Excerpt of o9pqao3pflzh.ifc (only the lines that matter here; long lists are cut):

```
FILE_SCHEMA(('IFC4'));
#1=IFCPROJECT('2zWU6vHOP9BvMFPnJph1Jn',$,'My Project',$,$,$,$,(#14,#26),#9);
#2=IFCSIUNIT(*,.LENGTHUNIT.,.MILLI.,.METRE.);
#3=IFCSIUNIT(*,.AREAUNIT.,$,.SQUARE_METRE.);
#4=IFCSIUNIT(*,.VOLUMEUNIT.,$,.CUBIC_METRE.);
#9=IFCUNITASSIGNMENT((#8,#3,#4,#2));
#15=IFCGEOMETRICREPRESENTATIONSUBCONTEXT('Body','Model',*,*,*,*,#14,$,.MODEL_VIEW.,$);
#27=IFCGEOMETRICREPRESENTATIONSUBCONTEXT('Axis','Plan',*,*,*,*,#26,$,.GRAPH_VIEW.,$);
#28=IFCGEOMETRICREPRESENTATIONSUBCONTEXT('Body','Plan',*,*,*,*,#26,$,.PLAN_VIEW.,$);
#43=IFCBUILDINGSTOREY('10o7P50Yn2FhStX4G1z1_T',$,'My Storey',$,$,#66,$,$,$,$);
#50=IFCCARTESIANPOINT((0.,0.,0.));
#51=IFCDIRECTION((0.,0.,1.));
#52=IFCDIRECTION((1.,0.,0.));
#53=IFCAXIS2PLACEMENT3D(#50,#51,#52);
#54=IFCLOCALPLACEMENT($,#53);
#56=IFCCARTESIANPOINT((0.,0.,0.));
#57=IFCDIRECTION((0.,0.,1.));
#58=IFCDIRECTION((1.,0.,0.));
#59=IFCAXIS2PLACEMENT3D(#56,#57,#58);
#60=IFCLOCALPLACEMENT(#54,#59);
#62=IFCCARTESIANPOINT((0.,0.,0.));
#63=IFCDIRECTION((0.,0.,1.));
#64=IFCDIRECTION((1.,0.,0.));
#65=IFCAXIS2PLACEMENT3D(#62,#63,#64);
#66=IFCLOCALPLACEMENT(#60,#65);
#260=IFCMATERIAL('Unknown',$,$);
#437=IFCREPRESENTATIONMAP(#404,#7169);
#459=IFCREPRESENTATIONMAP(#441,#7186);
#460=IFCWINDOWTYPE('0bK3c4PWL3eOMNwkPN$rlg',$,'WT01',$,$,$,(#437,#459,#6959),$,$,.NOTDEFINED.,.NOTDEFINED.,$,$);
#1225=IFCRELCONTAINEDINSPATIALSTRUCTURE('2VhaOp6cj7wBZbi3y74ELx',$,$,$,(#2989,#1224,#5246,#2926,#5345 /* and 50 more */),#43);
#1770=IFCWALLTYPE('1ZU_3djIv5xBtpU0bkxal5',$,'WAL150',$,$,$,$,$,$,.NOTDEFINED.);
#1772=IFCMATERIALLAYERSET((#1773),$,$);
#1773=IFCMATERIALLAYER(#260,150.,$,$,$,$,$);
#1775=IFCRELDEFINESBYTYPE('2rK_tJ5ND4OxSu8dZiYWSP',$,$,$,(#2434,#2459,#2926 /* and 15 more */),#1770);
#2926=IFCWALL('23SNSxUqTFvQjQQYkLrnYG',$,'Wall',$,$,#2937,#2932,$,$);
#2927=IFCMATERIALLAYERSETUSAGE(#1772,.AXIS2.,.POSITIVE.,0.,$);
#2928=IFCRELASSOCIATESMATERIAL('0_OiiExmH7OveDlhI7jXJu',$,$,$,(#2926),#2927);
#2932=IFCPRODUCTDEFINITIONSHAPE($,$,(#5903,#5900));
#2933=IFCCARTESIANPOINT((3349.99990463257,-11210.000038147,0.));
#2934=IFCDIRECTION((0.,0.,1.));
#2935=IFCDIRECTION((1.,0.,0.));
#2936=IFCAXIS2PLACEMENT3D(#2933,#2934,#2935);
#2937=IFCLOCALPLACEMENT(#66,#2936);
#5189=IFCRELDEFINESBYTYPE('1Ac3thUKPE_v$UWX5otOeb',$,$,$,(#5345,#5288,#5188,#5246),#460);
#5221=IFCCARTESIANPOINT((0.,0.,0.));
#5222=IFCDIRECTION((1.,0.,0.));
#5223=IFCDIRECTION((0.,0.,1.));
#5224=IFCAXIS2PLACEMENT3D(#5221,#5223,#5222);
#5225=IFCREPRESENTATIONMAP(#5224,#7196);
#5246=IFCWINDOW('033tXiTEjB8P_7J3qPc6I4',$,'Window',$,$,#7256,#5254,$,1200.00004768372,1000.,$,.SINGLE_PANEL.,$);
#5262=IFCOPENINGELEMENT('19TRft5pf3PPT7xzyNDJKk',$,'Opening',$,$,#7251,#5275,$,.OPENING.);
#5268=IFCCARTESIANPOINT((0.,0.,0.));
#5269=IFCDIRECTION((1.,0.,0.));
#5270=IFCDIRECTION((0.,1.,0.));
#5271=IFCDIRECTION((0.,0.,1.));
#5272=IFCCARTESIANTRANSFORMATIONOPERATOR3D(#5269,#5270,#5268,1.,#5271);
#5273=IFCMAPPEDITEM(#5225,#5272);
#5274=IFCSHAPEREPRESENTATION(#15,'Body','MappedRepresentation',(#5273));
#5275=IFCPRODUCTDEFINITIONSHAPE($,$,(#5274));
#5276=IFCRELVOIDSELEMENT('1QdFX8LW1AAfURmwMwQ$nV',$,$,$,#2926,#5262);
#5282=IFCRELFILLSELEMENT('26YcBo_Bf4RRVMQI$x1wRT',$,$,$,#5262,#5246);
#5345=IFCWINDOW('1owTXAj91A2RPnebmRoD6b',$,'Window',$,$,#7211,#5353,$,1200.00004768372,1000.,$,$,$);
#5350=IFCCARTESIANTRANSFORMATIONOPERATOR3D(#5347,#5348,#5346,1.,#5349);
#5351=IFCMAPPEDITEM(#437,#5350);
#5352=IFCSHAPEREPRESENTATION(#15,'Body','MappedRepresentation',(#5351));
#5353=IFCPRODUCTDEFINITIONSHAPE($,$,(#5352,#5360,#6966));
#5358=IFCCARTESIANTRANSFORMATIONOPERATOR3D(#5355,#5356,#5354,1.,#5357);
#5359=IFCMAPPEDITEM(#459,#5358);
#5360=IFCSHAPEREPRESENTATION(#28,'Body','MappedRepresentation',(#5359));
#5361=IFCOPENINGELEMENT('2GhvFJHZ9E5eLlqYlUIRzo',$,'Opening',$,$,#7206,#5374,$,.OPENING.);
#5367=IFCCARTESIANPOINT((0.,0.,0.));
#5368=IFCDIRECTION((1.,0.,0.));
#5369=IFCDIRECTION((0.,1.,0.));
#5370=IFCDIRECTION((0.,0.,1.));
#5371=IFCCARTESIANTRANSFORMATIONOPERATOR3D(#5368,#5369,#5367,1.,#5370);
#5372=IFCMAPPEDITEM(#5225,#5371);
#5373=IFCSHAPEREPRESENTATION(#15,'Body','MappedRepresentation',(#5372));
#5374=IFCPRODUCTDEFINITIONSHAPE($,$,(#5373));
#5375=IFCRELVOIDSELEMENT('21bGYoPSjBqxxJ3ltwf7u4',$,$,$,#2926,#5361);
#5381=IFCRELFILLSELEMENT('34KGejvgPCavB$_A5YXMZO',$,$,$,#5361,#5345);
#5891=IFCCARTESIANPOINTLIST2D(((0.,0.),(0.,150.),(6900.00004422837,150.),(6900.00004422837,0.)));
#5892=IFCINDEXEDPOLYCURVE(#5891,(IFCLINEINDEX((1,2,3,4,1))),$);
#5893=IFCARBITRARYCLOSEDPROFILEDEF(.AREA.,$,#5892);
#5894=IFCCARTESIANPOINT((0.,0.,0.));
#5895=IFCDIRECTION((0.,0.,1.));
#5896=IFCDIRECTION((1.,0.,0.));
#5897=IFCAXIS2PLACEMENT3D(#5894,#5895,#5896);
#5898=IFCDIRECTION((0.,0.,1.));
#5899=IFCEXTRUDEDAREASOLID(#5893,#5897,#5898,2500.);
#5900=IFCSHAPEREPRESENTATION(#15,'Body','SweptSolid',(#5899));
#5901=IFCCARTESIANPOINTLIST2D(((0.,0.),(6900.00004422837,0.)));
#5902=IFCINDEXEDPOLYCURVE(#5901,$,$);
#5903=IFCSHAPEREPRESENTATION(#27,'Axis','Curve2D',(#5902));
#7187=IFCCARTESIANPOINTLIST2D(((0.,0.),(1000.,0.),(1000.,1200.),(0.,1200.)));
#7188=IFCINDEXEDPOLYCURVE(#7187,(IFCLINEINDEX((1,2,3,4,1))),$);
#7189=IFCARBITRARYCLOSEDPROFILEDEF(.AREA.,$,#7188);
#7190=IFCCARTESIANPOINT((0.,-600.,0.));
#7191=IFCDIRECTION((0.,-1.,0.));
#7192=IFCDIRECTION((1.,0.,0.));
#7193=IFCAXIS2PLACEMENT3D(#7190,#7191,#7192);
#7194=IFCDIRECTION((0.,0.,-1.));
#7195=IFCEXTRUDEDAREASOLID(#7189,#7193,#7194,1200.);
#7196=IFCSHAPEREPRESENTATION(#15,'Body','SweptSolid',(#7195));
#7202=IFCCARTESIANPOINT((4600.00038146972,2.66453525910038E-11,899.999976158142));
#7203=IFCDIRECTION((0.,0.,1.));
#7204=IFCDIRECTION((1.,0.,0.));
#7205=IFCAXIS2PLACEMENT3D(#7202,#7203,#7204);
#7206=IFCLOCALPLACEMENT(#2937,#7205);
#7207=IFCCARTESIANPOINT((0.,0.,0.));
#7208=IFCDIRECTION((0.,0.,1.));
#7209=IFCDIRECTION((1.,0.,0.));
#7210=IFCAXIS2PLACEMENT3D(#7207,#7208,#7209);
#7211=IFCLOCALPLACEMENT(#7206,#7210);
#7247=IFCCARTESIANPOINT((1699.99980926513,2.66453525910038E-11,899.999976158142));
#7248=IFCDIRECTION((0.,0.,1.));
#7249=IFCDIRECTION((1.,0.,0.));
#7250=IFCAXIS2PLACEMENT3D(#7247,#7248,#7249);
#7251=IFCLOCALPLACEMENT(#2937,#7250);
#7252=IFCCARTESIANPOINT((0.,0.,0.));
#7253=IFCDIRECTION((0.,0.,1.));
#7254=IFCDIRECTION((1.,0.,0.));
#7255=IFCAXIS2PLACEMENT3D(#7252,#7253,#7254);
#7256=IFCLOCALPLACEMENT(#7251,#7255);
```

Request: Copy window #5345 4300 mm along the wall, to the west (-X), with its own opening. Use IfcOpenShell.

```python
import ifcopenshell
import ifcopenshell.api.feature
import ifcopenshell.api.geometry
import ifcopenshell.api.root
import ifcopenshell.geom
import ifcopenshell.util.element
import ifcopenshell.util.placement
import ifcopenshell.util.shape

model = ifcopenshell.open("o9pqao3pflzh.ifc")
settings = ifcopenshell.geom.settings()


def volume(element):
    """Net volume in cubic metres, openings subtracted."""
    shape = ifcopenshell.geom.create_shape(settings, element)
    return ifcopenshell.util.shape.get_volume(shape.geometry)


window = model.by_id(5345)
opening = window.FillsVoids[0].RelatingOpeningElement
wall = opening.VoidsElements[0].RelatingBuildingElement
before = volume(wall)
shift = ifcopenshell.util.placement.get_local_placement(wall.ObjectPlacement)[:3, 0] * -4300.0

# copy_class copies the void relationship, type, container and properties, but no geometry.
new_opening = ifcopenshell.api.root.copy_class(model, product=opening)
new_opening.Representation = ifcopenshell.util.element.copy_deep(
    model, opening.Representation, exclude=["IfcGeometricRepresentationContext", "IfcRepresentationMap"]
)
new_window = ifcopenshell.api.root.copy_class(model, product=window)
new_window.Representation = ifcopenshell.util.element.copy_deep(
    model, window.Representation, exclude=["IfcGeometricRepresentationContext", "IfcRepresentationMap"]
)
ifcopenshell.api.feature.add_filling(model, opening=new_opening, element=new_window)

for old, new in ((opening, new_opening), (window, new_window)):
    matrix = ifcopenshell.util.placement.get_local_placement(old.ObjectPlacement)
    matrix[:3, 3] += shift
    ifcopenshell.api.geometry.edit_object_placement(model, product=new, matrix=matrix, is_si=False)

after = volume(wall)

print(f"wall volume {before:.3f} -> {after:.3f} m3")

model.write("o9pqao3pflzh_v2.ifc")
```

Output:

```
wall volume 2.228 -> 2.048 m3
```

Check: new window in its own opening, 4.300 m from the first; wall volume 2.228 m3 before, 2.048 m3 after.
